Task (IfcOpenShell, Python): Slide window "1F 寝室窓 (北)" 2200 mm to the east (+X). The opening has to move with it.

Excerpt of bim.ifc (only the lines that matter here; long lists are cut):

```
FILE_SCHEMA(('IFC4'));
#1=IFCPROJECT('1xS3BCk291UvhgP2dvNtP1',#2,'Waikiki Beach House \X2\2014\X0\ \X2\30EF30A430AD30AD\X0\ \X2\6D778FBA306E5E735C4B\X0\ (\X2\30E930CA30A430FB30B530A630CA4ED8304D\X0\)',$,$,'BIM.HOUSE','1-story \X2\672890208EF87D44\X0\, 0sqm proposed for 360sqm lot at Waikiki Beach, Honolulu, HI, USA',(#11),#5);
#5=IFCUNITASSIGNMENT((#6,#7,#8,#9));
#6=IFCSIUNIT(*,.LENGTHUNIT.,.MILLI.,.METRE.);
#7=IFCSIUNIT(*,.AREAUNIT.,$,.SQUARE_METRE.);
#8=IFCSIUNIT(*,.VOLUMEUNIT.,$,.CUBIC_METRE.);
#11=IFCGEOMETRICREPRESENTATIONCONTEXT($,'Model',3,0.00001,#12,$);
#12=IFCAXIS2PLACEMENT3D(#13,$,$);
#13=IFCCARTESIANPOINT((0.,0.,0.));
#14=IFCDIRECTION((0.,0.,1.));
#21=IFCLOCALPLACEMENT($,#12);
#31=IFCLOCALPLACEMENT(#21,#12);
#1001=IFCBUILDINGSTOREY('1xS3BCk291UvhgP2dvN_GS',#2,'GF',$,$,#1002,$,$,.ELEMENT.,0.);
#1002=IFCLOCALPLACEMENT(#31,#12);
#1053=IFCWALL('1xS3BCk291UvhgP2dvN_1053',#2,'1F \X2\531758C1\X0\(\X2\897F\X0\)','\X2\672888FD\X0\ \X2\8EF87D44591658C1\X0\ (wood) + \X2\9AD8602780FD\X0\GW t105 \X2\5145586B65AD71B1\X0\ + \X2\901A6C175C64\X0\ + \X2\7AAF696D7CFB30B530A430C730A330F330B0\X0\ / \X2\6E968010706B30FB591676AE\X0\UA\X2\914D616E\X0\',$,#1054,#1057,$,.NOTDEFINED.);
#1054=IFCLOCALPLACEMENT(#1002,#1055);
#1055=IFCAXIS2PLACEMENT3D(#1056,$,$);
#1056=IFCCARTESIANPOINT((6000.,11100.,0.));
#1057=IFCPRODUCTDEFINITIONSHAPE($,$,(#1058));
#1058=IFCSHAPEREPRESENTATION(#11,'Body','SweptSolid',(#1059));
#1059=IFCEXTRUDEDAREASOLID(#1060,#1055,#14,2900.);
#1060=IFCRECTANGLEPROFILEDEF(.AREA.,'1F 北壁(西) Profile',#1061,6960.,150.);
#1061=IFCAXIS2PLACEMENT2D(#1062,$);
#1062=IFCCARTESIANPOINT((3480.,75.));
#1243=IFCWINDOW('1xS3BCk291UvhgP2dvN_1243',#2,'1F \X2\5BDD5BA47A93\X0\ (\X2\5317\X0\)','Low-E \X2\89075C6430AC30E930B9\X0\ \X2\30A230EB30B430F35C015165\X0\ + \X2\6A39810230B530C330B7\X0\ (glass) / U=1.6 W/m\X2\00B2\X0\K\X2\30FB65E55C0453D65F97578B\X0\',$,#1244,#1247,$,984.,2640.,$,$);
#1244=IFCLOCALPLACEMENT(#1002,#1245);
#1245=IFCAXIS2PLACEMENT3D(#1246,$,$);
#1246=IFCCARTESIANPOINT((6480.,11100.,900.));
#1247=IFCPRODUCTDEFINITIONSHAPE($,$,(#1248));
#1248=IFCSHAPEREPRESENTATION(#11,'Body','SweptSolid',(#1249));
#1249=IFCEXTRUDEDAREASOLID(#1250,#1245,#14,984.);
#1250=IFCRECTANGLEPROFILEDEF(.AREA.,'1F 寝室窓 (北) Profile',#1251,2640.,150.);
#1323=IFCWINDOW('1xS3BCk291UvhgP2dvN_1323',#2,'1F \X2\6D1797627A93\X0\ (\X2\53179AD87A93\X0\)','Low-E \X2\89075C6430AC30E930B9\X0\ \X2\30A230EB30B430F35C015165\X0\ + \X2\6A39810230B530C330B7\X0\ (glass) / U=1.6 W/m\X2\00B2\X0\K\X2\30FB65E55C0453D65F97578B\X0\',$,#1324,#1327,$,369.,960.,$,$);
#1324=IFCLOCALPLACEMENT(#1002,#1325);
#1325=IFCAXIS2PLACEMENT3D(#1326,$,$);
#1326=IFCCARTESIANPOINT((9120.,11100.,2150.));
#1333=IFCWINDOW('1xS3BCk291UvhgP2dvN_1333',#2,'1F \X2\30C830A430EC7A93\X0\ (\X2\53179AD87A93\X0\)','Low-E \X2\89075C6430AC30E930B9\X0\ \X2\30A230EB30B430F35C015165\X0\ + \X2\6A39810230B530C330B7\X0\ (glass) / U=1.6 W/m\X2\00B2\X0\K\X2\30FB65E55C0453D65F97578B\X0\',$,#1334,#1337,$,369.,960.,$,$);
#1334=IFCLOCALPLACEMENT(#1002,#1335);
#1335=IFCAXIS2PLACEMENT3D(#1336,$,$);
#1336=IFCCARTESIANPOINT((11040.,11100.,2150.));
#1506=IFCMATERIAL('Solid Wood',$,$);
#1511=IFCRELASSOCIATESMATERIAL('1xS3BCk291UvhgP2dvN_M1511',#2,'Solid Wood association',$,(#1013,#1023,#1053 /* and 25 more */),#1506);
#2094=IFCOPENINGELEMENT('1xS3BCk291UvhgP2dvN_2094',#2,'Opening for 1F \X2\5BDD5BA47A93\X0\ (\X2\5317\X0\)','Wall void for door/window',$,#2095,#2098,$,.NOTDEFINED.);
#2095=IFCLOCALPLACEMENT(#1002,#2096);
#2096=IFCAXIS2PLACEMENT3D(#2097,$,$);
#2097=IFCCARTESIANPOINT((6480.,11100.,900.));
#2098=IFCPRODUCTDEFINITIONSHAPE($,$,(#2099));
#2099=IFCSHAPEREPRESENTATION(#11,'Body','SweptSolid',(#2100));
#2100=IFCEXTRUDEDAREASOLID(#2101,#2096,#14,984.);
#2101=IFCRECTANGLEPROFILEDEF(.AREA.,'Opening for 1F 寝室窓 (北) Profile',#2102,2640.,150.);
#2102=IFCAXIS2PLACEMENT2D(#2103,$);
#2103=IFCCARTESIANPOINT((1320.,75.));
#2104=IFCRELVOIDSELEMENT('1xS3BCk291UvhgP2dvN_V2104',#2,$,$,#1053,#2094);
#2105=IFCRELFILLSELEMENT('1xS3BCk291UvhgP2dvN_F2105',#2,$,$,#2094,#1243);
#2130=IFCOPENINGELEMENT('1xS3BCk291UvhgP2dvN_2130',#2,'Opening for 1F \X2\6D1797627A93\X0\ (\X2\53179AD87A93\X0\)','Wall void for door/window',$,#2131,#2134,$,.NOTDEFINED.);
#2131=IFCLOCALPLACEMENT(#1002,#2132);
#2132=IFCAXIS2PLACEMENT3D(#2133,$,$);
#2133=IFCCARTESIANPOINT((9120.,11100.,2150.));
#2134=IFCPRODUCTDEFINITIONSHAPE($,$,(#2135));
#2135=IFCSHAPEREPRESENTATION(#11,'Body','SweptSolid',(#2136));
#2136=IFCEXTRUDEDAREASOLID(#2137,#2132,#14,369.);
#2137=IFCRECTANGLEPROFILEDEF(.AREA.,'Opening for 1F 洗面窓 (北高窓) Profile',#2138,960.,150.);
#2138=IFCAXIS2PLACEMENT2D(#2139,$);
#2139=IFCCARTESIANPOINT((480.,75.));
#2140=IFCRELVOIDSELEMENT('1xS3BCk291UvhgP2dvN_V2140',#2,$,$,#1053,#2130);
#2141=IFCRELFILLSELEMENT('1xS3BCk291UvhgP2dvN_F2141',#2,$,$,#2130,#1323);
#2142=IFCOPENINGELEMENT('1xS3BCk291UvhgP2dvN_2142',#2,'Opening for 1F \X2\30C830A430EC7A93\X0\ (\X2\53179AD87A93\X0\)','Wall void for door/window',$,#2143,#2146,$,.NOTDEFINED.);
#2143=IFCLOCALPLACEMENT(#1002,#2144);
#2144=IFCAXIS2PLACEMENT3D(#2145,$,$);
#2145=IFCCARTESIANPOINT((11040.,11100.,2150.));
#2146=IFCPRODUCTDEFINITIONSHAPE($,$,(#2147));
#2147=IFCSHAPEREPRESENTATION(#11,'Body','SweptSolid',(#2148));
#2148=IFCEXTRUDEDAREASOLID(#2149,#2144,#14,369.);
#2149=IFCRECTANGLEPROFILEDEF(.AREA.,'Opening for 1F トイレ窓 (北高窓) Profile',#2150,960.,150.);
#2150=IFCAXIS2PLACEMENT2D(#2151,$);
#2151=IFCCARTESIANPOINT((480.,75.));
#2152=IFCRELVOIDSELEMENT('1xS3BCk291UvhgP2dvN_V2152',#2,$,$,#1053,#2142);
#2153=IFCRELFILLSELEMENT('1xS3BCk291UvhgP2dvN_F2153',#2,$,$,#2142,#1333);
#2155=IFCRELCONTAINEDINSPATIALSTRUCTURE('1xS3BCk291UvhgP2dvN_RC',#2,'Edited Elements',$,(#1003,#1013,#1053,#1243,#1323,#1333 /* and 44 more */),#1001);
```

```python
import ifcopenshell
import ifcopenshell.api.geometry
import ifcopenshell.util.placement

model = ifcopenshell.open("bim.ifc")

window = model.by_guid("1xS3BCk291UvhgP2dvN_1243")
opening = window.FillsVoids[0].RelatingOpeningElement
wall = opening.VoidsElements[0].RelatingBuildingElement

wall_matrix = ifcopenshell.util.placement.get_local_placement(wall.ObjectPlacement)
shift = wall_matrix[:3, 0] * 2200.0
before = ifcopenshell.util.placement.get_local_placement(window.ObjectPlacement)[:3, 3].copy()

# The window is not placed relative to its opening, so move both.
for product in (opening, window):
    matrix = ifcopenshell.util.placement.get_local_placement(product.ObjectPlacement)
    matrix[:3, 3] += shift
    ifcopenshell.api.geometry.edit_object_placement(model, product=product, matrix=matrix, is_si=False)

after = ifcopenshell.util.placement.get_local_placement(window.ObjectPlacement)[:3, 3]
print("window moved by", (after - before).round(3) + 0.0)

model.write("bim_edited.ifc")
```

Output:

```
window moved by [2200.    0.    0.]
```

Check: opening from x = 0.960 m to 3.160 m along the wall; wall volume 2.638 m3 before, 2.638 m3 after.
